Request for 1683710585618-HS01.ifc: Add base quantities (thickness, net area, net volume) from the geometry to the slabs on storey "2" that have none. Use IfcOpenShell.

First a look at what the model holds.

```python
import ifcopenshell
import ifcopenshell.util.element
import ifcopenshell.util.unit

model = ifcopenshell.open("1683710585618-HS01.ifc")
print(model.schema)
for unit_type in ("LENGTHUNIT", "AREAUNIT", "VOLUMEUNIT"):
    print(unit_type, ifcopenshell.util.unit.calculate_unit_scale(model, unit_type))
storey = next(s for s in model.by_type("IfcBuildingStorey") if s.Name == "2")
slabs = [e for e in ifcopenshell.util.element.get_decomposition(storey) if e.is_a("IfcSlab")]
for e in sorted(slabs, key=lambda e: e.id()):
    print(e.id(), e.is_a(), e.Name, list(ifcopenshell.util.element.get_psets(e, qtos_only=True)), sep=" | ")
```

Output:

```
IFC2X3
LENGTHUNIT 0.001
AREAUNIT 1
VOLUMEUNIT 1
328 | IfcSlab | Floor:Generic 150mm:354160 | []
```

```python
import ifcopenshell
import ifcopenshell.api.pset
import ifcopenshell.geom
import ifcopenshell.util.element
import ifcopenshell.util.shape
import ifcopenshell.util.unit

model = ifcopenshell.open("1683710585618-HS01.ifc")
unit_scale = ifcopenshell.util.unit.calculate_unit_scale(model)
area_scale = ifcopenshell.util.unit.calculate_unit_scale(model, "AREAUNIT")
volume_scale = ifcopenshell.util.unit.calculate_unit_scale(model, "VOLUMEUNIT")
settings = ifcopenshell.geom.settings()

storey = next(s for s in model.by_type("IfcBuildingStorey") if s.Name == "2")
slabs = [e for e in ifcopenshell.util.element.get_decomposition(storey) if e.is_a("IfcSlab")]

for e in sorted(slabs, key=lambda e: e.id()):
    if ifcopenshell.util.element.get_psets(e, qtos_only=True, should_inherit=False):
        continue
    # Geometry comes back in metres, in the element's own axes.
    shape = ifcopenshell.geom.create_shape(settings, e)
    values = {
        "Width": ifcopenshell.util.shape.get_z(shape.geometry) / unit_scale,
        "NetArea": ifcopenshell.util.shape.get_footprint_area(shape.geometry) / area_scale,
        "NetVolume": ifcopenshell.util.shape.get_volume(shape.geometry) / volume_scale,
    }
    qto = ifcopenshell.api.pset.add_qto(model, product=e, name="BaseQuantities")
    ifcopenshell.api.pset.edit_qto(model, qto=qto, properties=values)
    print(e.id(), {k: round(v, 3) for k, v in values.items()})

model.write("1683710585618-HS01-out.ifc")
```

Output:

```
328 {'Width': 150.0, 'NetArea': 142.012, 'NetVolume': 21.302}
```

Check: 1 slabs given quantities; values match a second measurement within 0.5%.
